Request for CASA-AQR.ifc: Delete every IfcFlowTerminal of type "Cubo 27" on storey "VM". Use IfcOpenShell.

First a look at what the model holds.

```python
import ifcopenshell
import ifcopenshell.util.element

model = ifcopenshell.open("CASA-AQR.ifc")
print(model.schema)
storey = next(s for s in model.by_type("IfcBuildingStorey") if s.Name == "VM")
terminals = [e for e in ifcopenshell.util.element.get_decomposition(storey) if e.is_a("IfcFlowTerminal")]
seen = {}
for e in terminals:
    element_type = ifcopenshell.util.element.get_type(e)
    name = element_type.Name if element_type not in (None, e) else None
    seen[name] = seen.get(name, 0) + 1
for name, count in sorted(seen.items(), key=str):
    print(count, "x", name)
```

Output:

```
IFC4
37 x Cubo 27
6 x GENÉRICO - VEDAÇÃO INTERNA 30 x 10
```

```python
import ifcopenshell
import ifcopenshell.api.root
import ifcopenshell.util.element

model = ifcopenshell.open("CASA-AQR.ifc")

storey = next(s for s in model.by_type("IfcBuildingStorey") if s.Name == "VM")
terminals = [e for e in ifcopenshell.util.element.get_decomposition(storey) if e.is_a("IfcFlowTerminal")]
targets = [e for e in terminals if (t := ifcopenshell.util.element.get_type(e)) not in (None, e) and t.Name == "Cubo 27"]

for e in targets:
    ifcopenshell.api.root.remove_product(model, product=e)
print(len(targets), "removed")

model.write("CASA-AQR_rev.ifc")
```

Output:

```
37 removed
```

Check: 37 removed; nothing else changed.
